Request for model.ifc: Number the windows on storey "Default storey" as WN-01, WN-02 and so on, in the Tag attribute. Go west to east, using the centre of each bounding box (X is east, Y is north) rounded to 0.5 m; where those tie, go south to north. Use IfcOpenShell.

First a look at what the model holds.

```python
import ifcopenshell
import ifcopenshell.util.element
import ifcopenshell.util.placement

model = ifcopenshell.open("model.ifc")
print(model.schema)
storey = next(s for s in model.by_type("IfcBuildingStorey") if s.Name == "Default storey")
windows = [e for e in ifcopenshell.util.element.get_decomposition(storey) if e.is_a("IfcWindow")]
for e in sorted(windows, key=lambda e: e.id()):
    origin = ifcopenshell.util.placement.get_local_placement(e.ObjectPlacement)[:3, 3]
    print(e.id(), e.Tag, e.Name, origin.round(2) + 0.0, sep=" | ")
```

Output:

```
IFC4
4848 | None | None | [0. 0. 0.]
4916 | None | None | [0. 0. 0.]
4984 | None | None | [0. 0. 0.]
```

```python
import ifcopenshell
import ifcopenshell.geom
import ifcopenshell.util.element
import ifcopenshell.util.shape

model = ifcopenshell.open("model.ifc")
settings = ifcopenshell.geom.settings()
settings.set("use-world-coords", True)


def centre(element):
    shape = ifcopenshell.geom.create_shape(settings, element)
    return ifcopenshell.util.shape.get_bbox_centroid(shape.geometry)


storey = next(s for s in model.by_type("IfcBuildingStorey") if s.Name == "Default storey")
windows = [e for e in ifcopenshell.util.element.get_decomposition(storey) if e.is_a("IfcWindow")]

# Insertion points can sit at a corner or the storey origin, so sort by the geometry (in metres).
centres = {e: centre(e) for e in windows}
windows.sort(key=lambda e: (round(centres[e][0] / 0.5), centres[e][1]))

for i, e in enumerate(windows, start=1):
    number = f"WN-{i:02d}"
    e.Tag = number
    print(e.id(), number)

model.write("model_updated.ifc")
```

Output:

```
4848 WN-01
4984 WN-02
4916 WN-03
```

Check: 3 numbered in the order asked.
